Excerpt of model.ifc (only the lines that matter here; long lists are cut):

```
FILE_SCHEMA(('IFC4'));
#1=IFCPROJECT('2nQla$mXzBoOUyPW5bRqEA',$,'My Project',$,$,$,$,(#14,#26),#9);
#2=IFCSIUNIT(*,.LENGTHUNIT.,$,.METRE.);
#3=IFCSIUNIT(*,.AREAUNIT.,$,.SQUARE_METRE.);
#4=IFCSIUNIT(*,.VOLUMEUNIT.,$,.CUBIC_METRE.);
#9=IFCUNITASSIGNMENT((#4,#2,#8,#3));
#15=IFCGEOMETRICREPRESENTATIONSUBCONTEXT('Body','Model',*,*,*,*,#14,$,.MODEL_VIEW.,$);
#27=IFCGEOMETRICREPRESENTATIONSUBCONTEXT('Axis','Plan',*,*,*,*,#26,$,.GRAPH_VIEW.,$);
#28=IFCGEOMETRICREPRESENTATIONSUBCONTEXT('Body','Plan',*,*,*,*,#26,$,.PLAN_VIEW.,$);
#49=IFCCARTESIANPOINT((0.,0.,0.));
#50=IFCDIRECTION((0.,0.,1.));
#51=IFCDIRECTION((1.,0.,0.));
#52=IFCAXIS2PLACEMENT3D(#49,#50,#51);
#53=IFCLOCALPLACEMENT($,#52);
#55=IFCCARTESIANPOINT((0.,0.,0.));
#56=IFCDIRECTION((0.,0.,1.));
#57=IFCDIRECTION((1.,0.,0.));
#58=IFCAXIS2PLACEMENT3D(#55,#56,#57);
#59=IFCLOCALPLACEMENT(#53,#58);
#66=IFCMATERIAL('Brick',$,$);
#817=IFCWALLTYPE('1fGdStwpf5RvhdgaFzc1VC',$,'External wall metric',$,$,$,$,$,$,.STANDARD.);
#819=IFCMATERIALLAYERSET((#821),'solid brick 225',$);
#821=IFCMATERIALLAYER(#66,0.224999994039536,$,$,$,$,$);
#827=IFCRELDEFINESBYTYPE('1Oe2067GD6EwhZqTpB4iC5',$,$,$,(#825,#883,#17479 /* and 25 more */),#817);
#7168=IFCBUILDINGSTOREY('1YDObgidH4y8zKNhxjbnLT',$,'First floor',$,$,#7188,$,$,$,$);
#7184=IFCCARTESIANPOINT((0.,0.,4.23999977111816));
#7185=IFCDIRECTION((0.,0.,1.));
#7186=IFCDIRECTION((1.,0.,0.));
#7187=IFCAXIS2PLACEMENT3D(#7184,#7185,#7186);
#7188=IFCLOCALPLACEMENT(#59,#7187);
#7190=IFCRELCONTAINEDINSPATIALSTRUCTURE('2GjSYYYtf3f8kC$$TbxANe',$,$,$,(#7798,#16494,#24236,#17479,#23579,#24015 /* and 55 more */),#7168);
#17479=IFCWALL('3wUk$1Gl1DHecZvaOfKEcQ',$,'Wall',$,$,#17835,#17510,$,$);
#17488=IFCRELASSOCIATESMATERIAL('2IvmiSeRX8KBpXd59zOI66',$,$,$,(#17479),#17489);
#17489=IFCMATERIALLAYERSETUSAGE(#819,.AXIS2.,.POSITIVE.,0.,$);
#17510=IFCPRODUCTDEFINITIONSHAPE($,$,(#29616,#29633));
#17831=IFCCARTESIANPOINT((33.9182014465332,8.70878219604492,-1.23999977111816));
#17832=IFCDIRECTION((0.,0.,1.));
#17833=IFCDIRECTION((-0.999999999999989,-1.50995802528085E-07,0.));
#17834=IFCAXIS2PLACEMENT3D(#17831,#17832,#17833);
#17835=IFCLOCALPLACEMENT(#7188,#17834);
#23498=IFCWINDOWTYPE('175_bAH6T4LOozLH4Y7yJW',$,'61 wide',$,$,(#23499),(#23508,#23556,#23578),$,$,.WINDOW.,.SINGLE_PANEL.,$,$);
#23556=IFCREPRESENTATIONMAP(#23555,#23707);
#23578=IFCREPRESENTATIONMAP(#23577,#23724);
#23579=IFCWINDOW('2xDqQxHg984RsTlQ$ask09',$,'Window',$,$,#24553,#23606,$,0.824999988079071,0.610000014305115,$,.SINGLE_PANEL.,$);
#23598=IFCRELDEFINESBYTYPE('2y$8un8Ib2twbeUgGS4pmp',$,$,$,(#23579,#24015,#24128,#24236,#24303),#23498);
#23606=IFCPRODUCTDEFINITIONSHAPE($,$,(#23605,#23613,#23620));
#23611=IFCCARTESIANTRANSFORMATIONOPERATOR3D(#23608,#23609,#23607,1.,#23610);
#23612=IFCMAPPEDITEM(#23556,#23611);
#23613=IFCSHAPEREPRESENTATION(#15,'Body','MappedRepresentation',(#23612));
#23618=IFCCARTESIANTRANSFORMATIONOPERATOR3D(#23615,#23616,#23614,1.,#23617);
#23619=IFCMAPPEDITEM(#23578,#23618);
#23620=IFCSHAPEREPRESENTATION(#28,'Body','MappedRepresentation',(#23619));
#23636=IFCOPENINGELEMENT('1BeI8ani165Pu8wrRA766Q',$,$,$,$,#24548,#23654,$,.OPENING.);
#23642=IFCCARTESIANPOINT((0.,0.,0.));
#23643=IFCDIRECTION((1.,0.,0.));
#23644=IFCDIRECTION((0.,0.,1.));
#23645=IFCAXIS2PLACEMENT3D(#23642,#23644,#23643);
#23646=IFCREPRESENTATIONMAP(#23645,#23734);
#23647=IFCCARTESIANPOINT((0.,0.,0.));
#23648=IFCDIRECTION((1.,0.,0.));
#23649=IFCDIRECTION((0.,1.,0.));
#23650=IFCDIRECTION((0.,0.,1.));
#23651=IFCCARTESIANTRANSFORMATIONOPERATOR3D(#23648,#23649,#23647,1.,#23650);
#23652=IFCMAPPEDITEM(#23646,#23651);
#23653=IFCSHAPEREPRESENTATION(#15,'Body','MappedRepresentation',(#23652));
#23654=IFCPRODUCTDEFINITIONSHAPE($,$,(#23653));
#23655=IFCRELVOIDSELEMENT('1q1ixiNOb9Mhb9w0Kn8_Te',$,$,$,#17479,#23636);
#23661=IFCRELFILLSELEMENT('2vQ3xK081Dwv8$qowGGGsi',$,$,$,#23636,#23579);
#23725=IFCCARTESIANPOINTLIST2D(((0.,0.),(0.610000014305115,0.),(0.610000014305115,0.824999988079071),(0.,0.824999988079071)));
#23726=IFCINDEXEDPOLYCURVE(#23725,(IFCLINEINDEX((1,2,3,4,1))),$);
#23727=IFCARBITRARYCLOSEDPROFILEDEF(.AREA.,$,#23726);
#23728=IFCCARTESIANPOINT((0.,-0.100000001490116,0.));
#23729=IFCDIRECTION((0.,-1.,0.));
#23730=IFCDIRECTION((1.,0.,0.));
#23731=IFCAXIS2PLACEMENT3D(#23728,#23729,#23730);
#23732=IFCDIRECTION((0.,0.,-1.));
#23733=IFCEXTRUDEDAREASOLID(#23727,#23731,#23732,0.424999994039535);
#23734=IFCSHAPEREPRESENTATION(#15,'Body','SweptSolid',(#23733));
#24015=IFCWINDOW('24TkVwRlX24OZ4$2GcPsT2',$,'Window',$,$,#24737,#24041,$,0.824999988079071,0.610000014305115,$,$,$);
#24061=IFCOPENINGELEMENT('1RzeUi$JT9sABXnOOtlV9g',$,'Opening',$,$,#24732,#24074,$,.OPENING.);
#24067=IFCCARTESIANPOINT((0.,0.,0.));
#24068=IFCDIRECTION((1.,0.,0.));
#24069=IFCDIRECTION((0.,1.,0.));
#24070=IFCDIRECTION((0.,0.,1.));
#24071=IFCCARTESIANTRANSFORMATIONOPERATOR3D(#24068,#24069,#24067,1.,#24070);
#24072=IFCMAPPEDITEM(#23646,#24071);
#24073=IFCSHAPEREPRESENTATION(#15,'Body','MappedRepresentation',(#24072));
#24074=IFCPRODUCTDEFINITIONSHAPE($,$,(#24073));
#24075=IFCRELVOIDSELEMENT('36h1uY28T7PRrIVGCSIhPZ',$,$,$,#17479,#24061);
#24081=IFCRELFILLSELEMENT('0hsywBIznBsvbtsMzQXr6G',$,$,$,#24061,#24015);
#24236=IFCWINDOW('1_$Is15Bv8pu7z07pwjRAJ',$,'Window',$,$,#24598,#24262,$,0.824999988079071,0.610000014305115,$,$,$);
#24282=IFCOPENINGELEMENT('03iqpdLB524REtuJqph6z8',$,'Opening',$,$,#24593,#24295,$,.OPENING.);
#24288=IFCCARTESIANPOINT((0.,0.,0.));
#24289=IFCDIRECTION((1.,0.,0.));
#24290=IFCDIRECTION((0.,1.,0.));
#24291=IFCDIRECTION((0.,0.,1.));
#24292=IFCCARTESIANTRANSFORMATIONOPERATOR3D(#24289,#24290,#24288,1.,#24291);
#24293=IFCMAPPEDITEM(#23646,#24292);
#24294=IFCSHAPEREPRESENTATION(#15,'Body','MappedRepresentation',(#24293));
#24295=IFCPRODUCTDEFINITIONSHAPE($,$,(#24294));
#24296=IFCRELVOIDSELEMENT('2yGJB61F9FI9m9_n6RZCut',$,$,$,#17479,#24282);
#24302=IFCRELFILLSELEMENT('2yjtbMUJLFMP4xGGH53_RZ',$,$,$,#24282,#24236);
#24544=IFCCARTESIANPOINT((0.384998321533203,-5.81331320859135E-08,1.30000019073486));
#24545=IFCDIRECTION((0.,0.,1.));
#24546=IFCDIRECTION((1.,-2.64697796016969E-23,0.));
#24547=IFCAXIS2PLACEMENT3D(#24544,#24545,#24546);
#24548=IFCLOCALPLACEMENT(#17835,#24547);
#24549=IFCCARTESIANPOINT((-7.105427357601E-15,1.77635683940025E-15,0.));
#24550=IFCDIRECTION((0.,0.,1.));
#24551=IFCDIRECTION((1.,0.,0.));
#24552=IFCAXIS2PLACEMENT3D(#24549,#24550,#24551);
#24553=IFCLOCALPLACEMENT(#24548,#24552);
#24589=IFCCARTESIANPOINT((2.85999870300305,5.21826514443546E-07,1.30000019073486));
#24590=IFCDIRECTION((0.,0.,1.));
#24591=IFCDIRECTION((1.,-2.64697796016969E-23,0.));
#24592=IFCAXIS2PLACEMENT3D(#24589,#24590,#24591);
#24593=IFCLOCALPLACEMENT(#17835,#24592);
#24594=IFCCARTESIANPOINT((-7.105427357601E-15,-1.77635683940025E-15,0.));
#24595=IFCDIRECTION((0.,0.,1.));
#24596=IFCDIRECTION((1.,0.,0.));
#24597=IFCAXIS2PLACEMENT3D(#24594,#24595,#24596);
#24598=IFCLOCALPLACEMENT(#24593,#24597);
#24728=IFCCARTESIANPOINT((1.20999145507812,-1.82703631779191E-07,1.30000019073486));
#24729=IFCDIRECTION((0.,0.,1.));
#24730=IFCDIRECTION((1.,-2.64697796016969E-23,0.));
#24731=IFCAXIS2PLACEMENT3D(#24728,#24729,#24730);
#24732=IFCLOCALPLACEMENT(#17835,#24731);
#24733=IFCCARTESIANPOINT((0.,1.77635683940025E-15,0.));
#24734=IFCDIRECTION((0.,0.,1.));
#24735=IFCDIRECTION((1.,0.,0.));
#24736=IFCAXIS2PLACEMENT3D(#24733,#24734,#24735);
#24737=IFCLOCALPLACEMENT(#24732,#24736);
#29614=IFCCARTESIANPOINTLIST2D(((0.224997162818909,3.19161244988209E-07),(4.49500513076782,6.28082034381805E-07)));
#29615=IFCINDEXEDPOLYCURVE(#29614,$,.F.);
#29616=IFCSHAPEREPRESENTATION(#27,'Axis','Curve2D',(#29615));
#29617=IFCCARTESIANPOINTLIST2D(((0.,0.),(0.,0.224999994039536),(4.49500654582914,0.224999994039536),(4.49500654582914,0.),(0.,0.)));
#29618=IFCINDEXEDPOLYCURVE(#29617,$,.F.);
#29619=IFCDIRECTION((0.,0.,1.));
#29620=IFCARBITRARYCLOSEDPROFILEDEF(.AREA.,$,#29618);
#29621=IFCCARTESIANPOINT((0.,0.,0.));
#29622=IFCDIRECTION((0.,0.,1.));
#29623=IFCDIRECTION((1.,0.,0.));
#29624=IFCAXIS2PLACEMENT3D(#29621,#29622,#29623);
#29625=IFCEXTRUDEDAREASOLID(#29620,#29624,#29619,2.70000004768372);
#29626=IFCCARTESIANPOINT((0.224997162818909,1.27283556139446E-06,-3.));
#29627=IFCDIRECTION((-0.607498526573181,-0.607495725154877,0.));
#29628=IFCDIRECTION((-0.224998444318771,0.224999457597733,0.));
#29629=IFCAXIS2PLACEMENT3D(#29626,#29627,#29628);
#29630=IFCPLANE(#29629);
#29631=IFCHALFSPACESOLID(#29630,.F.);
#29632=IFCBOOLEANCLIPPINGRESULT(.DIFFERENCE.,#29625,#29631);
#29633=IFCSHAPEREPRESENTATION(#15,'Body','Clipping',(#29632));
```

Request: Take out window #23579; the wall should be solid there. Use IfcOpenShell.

```python
import ifcopenshell
import ifcopenshell.api.feature
import ifcopenshell.api.root
import ifcopenshell.geom
import ifcopenshell.util.shape

model = ifcopenshell.open("model.ifc")
settings = ifcopenshell.geom.settings()


def volume(element):
    """Net volume in cubic metres, openings subtracted."""
    shape = ifcopenshell.geom.create_shape(settings, element)
    return ifcopenshell.util.shape.get_volume(shape.geometry)


window = model.by_guid("2xDqQxHg984RsTlQ$ask09")
opening = window.FillsVoids[0].RelatingOpeningElement
wall = opening.VoidsElements[0].RelatingBuildingElement
before = volume(wall)

ifcopenshell.api.root.remove_product(model, product=window)
ifcopenshell.api.feature.remove_feature(model, feature=opening)

after = volume(wall)

print(f"wall volume {before:.3f} -> {after:.3f} m3")

model.write("model_updated.ifc")
```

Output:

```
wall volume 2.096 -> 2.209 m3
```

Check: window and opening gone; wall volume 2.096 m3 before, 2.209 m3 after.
